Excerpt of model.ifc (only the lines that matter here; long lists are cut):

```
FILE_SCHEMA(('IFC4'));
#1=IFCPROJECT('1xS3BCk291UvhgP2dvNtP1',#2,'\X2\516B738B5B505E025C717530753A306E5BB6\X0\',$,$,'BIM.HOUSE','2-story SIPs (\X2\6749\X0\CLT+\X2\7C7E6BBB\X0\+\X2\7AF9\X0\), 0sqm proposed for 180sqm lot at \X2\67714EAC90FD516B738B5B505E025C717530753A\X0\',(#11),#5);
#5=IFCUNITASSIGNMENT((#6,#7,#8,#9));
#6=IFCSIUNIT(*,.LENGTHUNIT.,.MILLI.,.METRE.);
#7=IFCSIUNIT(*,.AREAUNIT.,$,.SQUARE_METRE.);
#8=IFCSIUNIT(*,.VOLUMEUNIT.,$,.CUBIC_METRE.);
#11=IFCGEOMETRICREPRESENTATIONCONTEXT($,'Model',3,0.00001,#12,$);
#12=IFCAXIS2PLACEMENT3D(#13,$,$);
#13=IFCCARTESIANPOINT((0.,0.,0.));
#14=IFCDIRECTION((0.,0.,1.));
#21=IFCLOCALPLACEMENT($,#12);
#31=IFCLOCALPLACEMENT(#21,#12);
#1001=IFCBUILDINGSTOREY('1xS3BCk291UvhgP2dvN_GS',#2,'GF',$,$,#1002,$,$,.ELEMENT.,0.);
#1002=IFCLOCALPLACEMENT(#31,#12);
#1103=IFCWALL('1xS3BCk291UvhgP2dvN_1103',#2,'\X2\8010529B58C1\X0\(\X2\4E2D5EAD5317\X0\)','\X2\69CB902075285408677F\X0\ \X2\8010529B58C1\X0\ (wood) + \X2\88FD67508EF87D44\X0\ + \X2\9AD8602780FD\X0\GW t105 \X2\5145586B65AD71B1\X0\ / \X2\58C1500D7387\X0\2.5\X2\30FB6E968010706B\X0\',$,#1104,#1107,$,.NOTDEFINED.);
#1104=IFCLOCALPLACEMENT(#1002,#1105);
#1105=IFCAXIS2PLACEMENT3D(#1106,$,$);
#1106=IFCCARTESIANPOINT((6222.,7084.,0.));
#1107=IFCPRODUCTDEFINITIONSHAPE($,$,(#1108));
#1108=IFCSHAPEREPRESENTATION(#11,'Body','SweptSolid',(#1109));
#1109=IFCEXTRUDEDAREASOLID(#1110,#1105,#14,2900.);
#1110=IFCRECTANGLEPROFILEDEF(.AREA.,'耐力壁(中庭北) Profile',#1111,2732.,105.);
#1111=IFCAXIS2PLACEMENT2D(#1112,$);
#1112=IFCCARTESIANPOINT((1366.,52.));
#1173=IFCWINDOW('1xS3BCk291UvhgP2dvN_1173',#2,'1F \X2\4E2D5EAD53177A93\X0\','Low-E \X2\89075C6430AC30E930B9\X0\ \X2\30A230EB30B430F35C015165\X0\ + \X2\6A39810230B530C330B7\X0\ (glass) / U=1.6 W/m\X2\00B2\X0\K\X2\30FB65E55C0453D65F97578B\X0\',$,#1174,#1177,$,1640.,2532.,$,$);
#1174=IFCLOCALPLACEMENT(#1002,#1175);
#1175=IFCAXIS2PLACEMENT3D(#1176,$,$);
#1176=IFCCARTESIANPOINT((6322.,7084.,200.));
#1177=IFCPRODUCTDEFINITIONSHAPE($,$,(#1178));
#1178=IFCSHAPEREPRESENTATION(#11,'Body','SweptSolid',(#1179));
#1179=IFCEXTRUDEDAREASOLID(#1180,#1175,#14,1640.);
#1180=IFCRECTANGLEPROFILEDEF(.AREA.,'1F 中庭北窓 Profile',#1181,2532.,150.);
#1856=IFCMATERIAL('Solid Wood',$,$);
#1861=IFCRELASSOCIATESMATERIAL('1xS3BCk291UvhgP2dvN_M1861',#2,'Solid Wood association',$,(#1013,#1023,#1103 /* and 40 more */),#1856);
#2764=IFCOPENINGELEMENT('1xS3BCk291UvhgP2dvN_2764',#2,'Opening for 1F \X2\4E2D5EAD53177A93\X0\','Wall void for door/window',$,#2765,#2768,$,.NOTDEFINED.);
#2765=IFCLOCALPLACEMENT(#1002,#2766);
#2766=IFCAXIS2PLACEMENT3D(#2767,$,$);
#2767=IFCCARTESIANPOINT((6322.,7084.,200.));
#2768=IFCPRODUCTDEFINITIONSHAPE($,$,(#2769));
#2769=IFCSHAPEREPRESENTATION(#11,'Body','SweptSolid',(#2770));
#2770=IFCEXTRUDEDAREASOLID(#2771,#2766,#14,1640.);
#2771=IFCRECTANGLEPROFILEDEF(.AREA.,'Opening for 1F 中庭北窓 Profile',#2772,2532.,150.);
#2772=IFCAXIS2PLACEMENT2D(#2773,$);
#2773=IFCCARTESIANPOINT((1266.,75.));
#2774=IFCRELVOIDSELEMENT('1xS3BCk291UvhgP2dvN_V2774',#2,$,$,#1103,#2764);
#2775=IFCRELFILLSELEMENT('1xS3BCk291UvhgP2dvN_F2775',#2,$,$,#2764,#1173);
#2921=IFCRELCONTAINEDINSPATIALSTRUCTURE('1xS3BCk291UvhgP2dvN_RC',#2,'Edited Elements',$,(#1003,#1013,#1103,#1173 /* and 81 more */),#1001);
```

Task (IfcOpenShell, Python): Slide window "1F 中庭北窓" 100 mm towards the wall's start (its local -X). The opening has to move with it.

```python
import ifcopenshell
import ifcopenshell.api.geometry
import ifcopenshell.util.placement

model = ifcopenshell.open("model.ifc")

window = model.by_id(1173)
opening = window.FillsVoids[0].RelatingOpeningElement
wall = opening.VoidsElements[0].RelatingBuildingElement

wall_matrix = ifcopenshell.util.placement.get_local_placement(wall.ObjectPlacement)
shift = wall_matrix[:3, 0] * -100.0
before = ifcopenshell.util.placement.get_local_placement(window.ObjectPlacement)[:3, 3].copy()

# The window is not placed relative to its opening, so move both.
for product in (opening, window):
    matrix = ifcopenshell.util.placement.get_local_placement(product.ObjectPlacement)
    matrix[:3, 3] += shift
    ifcopenshell.api.geometry.edit_object_placement(model, product=product, matrix=matrix, is_si=False)

after = ifcopenshell.util.placement.get_local_placement(window.ObjectPlacement)[:3, 3]
print("window moved by", (after - before).round(3) + 0.0)

model.write("model_rev.ifc")
```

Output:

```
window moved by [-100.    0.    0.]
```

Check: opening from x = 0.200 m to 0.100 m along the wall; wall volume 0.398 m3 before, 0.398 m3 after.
